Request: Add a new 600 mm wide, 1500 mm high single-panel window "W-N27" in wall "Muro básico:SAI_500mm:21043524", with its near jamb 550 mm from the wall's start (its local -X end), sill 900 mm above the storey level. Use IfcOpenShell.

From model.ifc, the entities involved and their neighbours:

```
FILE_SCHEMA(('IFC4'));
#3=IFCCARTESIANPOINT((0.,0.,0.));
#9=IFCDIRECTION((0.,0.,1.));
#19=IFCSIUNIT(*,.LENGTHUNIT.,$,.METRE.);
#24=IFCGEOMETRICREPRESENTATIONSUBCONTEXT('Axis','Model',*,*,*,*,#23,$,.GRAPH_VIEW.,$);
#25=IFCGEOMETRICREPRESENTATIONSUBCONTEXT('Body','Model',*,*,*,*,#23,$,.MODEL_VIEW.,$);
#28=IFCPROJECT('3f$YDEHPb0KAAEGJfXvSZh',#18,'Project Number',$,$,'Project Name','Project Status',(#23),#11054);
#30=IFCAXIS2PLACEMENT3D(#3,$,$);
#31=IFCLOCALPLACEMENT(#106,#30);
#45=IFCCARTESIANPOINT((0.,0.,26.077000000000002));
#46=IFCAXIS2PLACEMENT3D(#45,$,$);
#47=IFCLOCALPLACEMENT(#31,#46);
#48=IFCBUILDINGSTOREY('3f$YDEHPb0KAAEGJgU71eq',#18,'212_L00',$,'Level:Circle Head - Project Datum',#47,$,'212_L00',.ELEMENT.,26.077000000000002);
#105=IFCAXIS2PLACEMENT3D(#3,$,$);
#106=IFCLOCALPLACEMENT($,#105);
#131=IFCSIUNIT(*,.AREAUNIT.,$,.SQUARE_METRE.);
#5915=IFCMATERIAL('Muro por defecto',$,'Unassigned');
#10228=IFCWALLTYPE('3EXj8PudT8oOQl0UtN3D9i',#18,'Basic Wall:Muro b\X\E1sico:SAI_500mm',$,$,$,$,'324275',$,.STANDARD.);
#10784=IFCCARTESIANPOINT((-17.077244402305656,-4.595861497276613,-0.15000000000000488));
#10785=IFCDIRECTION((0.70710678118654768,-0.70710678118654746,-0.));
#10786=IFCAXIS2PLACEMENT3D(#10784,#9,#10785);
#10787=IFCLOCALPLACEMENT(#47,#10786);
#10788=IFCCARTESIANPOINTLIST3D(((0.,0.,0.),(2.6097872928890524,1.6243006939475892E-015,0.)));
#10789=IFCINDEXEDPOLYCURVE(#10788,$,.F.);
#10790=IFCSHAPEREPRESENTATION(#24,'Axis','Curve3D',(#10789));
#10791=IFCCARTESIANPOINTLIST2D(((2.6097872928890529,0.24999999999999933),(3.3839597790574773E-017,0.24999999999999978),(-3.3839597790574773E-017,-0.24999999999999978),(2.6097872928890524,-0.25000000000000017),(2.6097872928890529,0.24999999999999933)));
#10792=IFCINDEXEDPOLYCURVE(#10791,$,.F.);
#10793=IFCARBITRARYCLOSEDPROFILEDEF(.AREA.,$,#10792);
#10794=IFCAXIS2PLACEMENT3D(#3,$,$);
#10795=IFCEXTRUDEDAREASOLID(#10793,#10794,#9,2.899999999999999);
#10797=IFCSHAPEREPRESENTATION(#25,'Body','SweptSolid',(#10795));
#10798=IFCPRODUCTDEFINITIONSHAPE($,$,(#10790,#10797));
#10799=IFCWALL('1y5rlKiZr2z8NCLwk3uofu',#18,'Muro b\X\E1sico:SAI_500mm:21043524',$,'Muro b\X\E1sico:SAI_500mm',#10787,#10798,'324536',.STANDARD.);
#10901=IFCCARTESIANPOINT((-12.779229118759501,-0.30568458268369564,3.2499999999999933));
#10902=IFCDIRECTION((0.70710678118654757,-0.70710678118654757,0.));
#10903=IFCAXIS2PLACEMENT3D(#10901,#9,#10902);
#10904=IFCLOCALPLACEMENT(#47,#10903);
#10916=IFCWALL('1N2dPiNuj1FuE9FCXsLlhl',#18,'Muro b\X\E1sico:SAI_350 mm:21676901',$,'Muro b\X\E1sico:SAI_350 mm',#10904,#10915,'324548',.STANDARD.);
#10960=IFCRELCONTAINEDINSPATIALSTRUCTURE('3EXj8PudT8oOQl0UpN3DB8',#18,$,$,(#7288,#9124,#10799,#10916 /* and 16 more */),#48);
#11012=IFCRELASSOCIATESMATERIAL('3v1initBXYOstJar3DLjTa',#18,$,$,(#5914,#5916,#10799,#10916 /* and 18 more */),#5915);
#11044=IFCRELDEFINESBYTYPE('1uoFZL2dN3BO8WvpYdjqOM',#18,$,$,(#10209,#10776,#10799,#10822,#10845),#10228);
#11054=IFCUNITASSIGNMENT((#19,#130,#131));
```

```python
import numpy as np
import ifcopenshell
import ifcopenshell.api.feature
import ifcopenshell.api.geometry
import ifcopenshell.api.root
import ifcopenshell.api.spatial
import ifcopenshell.geom
import ifcopenshell.util.element
import ifcopenshell.util.placement
import ifcopenshell.util.representation
import ifcopenshell.util.shape
import ifcopenshell.util.unit

model = ifcopenshell.open("model.ifc")
unit_scale = ifcopenshell.util.unit.calculate_unit_scale(model)
settings = ifcopenshell.geom.settings()


def volume(element):
    """Net volume in cubic metres, openings subtracted."""
    shape = ifcopenshell.geom.create_shape(settings, element)
    return ifcopenshell.util.shape.get_volume(shape.geometry)


wall = model.by_id(10799)
storey = ifcopenshell.util.element.get_container(wall, ifc_class="IfcBuildingStorey")
context = ifcopenshell.util.representation.get_context(model, "Model", "Body", "MODEL_VIEW")
before = volume(wall)

width, height, from_end, sill = 0.6, 1.5, 0.55, 0.9  # metres

# The wall runs along its own X axis, and the end named is its -X end.
wall_shape = ifcopenshell.geom.create_shape(settings, wall)
x, y, z = ifcopenshell.util.shape.get_vertices(wall_shape.geometry).T
start = x.min() + from_end
face, thickness = float(y.min()), float(y.max() - y.min())
wall_matrix = ifcopenshell.util.placement.get_local_placement(wall.ObjectPlacement)
level = ifcopenshell.util.placement.get_local_placement(storey.ObjectPlacement)[2, 3]


def in_wall(x, y):
    """Placement at x, y metres in the wall's axes, at sill height."""
    matrix = wall_matrix.copy()
    matrix[:, 3] = wall_matrix @ np.array([x / unit_scale, y / unit_scale, 0.0, 1.0])
    matrix[2, 3] = level + sill / unit_scale
    return matrix


# Opening: a box that overshoots both wall faces by 50 mm.
opening = ifcopenshell.api.root.create_entity(model, ifc_class="IfcOpeningElement", predefined_type="OPENING")
box = ifcopenshell.api.geometry.add_wall_representation(
    model, context=context, length=width, height=height, thickness=thickness + 0.1
)
ifcopenshell.api.geometry.assign_representation(model, product=opening, representation=box)
ifcopenshell.api.geometry.edit_object_placement(model, product=opening, matrix=in_wall(start, face - 0.05), is_si=False)
ifcopenshell.api.feature.add_feature(model, feature=opening, element=wall)

window = ifcopenshell.api.root.create_entity(model, ifc_class="IfcWindow", name="W-N27", predefined_type="WINDOW")
window.OverallWidth, window.OverallHeight = width / unit_scale, height / unit_scale
window.PartitioningType = "SINGLE_PANEL"
body = ifcopenshell.api.geometry.add_window_representation(
    model,
    context=context,
    overall_width=window.OverallWidth,
    overall_height=window.OverallHeight,
    partition_type="SINGLE_PANEL",
)
ifcopenshell.api.geometry.assign_representation(model, product=window, representation=body)
ifcopenshell.api.spatial.assign_container(model, products=[window], relating_structure=storey)
ifcopenshell.api.feature.add_filling(model, opening=opening, element=window)

# Centre the window in the wall's thickness.
ifcopenshell.api.geometry.edit_object_placement(model, product=window, matrix=in_wall(start, face), is_si=False)
window_shape = ifcopenshell.geom.create_shape(settings, window)
depth = ifcopenshell.util.shape.get_vertices(window_shape.geometry)[:, 1]
offset = face + thickness / 2 - (depth.min() + depth.max()) / 2
ifcopenshell.api.geometry.edit_object_placement(model, product=window, matrix=in_wall(start, offset), is_si=False)

after = volume(wall)

print(f"wall volume {before:.3f} -> {after:.3f} m3")

model.write("model_v2.ifc")
```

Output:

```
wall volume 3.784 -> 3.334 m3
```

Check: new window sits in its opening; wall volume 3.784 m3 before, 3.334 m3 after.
